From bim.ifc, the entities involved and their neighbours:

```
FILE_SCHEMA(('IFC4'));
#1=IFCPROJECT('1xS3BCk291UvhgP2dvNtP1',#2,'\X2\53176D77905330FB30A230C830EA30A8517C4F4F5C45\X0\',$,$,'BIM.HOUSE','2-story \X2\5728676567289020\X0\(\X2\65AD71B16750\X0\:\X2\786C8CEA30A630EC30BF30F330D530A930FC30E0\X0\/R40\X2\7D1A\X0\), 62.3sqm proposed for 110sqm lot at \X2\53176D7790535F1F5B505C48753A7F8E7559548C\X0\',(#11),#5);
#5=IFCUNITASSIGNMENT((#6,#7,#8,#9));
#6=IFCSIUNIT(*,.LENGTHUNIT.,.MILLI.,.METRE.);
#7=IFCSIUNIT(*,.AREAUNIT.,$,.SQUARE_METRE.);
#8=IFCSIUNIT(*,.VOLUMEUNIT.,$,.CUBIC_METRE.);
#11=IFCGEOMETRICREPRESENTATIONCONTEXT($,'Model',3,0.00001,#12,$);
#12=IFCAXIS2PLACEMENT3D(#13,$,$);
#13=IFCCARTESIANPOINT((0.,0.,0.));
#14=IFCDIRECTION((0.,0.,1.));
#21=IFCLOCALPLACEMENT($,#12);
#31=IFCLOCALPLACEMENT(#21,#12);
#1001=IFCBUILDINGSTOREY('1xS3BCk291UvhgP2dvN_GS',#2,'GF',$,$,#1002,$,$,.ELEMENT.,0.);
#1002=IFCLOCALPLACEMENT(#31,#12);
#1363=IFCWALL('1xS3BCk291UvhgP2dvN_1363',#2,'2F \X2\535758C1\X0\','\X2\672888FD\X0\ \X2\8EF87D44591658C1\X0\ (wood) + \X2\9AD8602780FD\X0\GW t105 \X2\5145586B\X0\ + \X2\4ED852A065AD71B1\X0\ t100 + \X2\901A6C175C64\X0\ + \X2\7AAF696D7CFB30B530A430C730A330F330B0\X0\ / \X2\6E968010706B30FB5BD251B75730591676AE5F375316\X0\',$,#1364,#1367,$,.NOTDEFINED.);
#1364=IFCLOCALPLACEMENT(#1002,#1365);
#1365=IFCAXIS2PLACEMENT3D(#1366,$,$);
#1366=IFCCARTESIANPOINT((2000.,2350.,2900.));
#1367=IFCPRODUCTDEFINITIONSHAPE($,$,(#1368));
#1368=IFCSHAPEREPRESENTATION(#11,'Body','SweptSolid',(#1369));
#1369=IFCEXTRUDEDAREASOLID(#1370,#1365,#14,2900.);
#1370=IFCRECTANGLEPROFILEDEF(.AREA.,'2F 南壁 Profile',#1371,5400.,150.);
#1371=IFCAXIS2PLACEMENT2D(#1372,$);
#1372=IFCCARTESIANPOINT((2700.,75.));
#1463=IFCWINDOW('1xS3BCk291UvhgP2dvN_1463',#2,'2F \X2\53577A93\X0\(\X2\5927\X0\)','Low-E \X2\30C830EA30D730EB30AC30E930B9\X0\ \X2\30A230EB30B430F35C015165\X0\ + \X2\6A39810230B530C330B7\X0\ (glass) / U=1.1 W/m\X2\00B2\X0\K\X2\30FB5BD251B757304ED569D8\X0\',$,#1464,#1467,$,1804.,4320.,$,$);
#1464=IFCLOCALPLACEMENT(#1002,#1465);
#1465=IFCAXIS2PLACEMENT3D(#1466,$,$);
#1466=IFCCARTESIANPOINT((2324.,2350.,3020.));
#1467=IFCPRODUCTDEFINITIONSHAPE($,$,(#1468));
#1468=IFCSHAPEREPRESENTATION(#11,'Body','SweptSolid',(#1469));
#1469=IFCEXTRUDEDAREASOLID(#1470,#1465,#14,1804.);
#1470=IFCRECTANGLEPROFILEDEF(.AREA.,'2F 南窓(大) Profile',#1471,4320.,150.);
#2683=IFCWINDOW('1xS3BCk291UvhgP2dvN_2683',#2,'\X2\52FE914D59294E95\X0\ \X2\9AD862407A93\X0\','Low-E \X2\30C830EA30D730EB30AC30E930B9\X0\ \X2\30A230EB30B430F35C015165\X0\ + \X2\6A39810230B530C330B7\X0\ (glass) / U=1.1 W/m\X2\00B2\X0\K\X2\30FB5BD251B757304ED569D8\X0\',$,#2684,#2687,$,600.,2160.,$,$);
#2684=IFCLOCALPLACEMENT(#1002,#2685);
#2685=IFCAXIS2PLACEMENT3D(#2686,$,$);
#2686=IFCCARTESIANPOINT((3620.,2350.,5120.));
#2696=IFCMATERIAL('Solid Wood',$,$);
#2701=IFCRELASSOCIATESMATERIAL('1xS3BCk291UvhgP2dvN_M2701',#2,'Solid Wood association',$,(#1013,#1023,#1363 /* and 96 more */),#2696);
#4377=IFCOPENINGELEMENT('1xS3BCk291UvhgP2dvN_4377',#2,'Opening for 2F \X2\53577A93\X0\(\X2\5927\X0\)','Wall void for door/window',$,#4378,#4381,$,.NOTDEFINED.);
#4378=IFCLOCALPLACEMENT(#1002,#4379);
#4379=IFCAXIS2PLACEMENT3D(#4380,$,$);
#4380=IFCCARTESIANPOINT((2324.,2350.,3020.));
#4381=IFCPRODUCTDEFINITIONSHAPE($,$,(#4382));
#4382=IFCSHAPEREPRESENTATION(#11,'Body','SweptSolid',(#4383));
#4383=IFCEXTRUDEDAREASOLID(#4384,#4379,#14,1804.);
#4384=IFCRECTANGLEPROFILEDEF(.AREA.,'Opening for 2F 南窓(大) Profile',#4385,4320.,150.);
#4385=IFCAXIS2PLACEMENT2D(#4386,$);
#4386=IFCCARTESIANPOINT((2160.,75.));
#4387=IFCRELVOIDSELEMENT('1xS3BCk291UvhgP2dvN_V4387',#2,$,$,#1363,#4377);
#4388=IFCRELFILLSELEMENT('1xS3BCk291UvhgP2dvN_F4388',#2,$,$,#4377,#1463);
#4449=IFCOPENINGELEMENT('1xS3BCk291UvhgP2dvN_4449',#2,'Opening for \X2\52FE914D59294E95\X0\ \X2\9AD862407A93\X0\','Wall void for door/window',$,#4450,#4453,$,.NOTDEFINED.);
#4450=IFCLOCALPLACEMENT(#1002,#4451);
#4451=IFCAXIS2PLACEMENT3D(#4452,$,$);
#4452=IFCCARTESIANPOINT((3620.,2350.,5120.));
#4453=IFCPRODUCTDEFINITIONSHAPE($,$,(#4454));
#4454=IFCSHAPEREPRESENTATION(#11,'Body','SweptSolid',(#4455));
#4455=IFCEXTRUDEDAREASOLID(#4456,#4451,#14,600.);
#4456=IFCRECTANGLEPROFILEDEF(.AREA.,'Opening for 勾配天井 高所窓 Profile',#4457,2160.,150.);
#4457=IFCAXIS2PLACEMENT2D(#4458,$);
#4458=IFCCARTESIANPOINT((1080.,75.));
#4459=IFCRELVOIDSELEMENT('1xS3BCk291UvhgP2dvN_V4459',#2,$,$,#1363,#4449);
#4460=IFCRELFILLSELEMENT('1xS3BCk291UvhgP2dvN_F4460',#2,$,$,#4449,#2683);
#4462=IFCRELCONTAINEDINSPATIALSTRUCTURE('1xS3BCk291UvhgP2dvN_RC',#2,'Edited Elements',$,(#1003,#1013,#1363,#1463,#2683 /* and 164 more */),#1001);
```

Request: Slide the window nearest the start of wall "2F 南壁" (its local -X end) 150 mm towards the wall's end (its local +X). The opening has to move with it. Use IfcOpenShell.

```python
import ifcopenshell
import ifcopenshell.api.geometry
import ifcopenshell.util.placement
import ifcopenshell.util.unit

model = ifcopenshell.open("bim.ifc")
unit_scale = ifcopenshell.util.unit.calculate_unit_scale(model)

window = model.by_guid("1xS3BCk291UvhgP2dvN_1463")
opening = window.FillsVoids[0].RelatingOpeningElement
wall = opening.VoidsElements[0].RelatingBuildingElement

wall_matrix = ifcopenshell.util.placement.get_local_placement(wall.ObjectPlacement)
shift = wall_matrix[:3, 0] * 0.15 / unit_scale
before = ifcopenshell.util.placement.get_local_placement(window.ObjectPlacement)[:3, 3].copy()

# The window is not placed relative to its opening, so move both.
for product in (opening, window):
    matrix = ifcopenshell.util.placement.get_local_placement(product.ObjectPlacement)
    matrix[:3, 3] += shift
    ifcopenshell.api.geometry.edit_object_placement(model, product=product, matrix=matrix, is_si=False)

after = ifcopenshell.util.placement.get_local_placement(window.ObjectPlacement)[:3, 3]
print("window moved by", (after - before).round(3) + 0.0)

model.write("bim_edited.ifc")
```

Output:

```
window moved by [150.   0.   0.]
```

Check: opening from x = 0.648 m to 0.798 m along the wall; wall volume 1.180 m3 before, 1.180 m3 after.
